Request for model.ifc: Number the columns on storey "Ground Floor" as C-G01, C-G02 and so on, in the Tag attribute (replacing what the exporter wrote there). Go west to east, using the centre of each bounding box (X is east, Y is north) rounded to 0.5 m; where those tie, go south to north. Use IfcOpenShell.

First a look at what the model holds.

```python
import ifcopenshell
import ifcopenshell.util.element
import ifcopenshell.util.placement

model = ifcopenshell.open("model.ifc")
print(model.schema)
storey = next(s for s in model.by_type("IfcBuildingStorey") if s.Name == "Ground Floor")
columns = [e for e in ifcopenshell.util.element.get_decomposition(storey) if e.is_a("IfcColumn")]
for e in sorted(columns, key=lambda e: e.id()):
    origin = ifcopenshell.util.placement.get_local_placement(e.ObjectPlacement)[:3, 3]
    print(e.id(), e.Tag, e.Name, origin.round(2) + 0.0, sep=" | ")
```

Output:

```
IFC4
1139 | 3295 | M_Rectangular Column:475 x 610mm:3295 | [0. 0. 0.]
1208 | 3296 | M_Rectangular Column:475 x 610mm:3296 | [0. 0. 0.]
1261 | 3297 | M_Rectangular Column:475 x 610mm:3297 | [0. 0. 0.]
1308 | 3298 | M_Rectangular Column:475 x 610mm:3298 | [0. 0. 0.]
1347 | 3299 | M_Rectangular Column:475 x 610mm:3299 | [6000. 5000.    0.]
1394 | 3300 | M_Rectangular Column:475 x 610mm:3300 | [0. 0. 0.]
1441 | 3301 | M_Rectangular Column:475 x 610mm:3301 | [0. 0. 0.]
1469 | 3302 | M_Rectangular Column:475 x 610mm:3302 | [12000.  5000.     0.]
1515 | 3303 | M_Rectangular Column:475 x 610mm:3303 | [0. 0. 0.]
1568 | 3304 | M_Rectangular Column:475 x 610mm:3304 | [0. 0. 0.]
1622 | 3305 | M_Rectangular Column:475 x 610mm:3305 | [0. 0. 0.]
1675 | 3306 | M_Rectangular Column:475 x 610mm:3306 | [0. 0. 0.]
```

```python
import ifcopenshell
import ifcopenshell.geom
import ifcopenshell.util.element
import ifcopenshell.util.shape

model = ifcopenshell.open("model.ifc")
settings = ifcopenshell.geom.settings()
settings.set("use-world-coords", True)


def centre(element):
    shape = ifcopenshell.geom.create_shape(settings, element)
    return ifcopenshell.util.shape.get_bbox_centroid(shape.geometry)


storey = next(s for s in model.by_type("IfcBuildingStorey") if s.Name == "Ground Floor")
columns = [e for e in ifcopenshell.util.element.get_decomposition(storey) if e.is_a("IfcColumn")]

# Insertion points can sit at a corner or the storey origin, so sort by the geometry (in metres).
centres = {e: centre(e) for e in columns}
columns.sort(key=lambda e: (round(centres[e][0] / 0.5), centres[e][1]))

for i, e in enumerate(columns, start=1):
    number = f"C-G{i:02d}"
    e.Tag = number
    print(e.id(), number)

model.write("model_edited.ifc")
```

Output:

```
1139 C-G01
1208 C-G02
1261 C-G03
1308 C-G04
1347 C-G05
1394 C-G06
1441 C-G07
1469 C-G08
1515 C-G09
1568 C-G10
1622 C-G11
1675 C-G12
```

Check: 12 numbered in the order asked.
